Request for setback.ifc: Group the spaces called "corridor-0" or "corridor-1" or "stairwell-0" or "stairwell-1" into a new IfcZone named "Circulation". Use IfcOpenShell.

First a look at what the model holds.

```python
import ifcopenshell

model = ifcopenshell.open("setback.ifc")
print(model.schema)
seen = {}
for space in model.by_type("IfcSpace"):
    seen[space.Name] = seen.get(space.Name, 0) + 1
for name, count in sorted(seen.items(), key=str):
    print(count, "x", name)
print("zones:", [z.Name for z in model.by_type("IfcZone")][:20])
```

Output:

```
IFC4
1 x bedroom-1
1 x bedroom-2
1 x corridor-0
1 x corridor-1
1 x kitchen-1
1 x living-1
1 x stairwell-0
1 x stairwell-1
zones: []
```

```python
import ifcopenshell
import ifcopenshell.api.group
import ifcopenshell.api.root

model = ifcopenshell.open("setback.ifc")

names = {"corridor-0", "corridor-1", "stairwell-0", "stairwell-1"}
spaces = [s for s in model.by_type("IfcSpace") if s.Name in names]

zone = ifcopenshell.api.root.create_entity(model, ifc_class="IfcZone", name="Circulation")
ifcopenshell.api.group.assign_group(model, products=spaces, group=zone)
print(len(spaces), "spaces in", zone.Name)

model.write("setback_edited.ifc")
```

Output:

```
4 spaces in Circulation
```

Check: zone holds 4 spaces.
